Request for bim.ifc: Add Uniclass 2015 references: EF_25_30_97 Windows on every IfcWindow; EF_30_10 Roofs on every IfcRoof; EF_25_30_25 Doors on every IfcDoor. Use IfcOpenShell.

First a look at what the model holds.

```python
import ifcopenshell

model = ifcopenshell.open("bim.ifc")
print(model.schema)
print("classifications:", [c.Name for c in model.by_type("IfcClassification")])
for ifc_class in ("IfcDoor", "IfcRoof", "IfcStair", "IfcWall", "IfcWindow"):
    print(ifc_class, len(model.by_type(ifc_class)))
```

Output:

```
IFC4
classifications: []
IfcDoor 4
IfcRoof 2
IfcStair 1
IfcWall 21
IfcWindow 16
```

```python
import ifcopenshell
import ifcopenshell.api.classification

model = ifcopenshell.open("bim.ifc")

system = ifcopenshell.api.classification.add_classification(model, classification="Uniclass 2015")

codes = {
    "IfcWindow": ("EF_25_30_97", "Windows"),
    "IfcRoof": ("EF_30_10", "Roofs"),
    "IfcDoor": ("EF_25_30_25", "Doors"),
}
for ifc_class, (code, name) in codes.items():
    products = model.by_type(ifc_class)
    ifcopenshell.api.classification.add_reference(
        model, products=products, classification=system, identification=code, name=name
    )
    print(code, len(products))

model.write("bim_updated.ifc")
```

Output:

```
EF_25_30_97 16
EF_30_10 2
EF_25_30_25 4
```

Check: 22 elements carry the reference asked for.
